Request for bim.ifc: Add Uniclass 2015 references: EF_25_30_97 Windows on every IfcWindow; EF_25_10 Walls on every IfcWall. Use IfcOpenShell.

First a look at what the model holds.

```python
import ifcopenshell

model = ifcopenshell.open("bim.ifc")
print(model.schema)
print("classifications:", [c.Name for c in model.by_type("IfcClassification")])
for ifc_class in ("IfcDoor", "IfcRoof", "IfcStair", "IfcWall", "IfcWindow"):
    print(ifc_class, len(model.by_type(ifc_class)))
```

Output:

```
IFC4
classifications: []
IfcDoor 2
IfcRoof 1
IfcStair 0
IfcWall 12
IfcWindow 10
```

```python
import ifcopenshell
import ifcopenshell.api.classification

model = ifcopenshell.open("bim.ifc")

system = ifcopenshell.api.classification.add_classification(model, classification="Uniclass 2015")

codes = {
    "IfcWindow": ("EF_25_30_97", "Windows"),
    "IfcWall": ("EF_25_10", "Walls"),
}
for ifc_class, (code, name) in codes.items():
    products = model.by_type(ifc_class)
    ifcopenshell.api.classification.add_reference(
        model, products=products, classification=system, identification=code, name=name
    )
    print(code, len(products))

model.write("bim_v2.ifc")
```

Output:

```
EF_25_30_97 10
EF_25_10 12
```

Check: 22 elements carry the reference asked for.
